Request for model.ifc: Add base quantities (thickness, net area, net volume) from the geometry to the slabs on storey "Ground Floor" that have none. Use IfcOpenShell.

First a look at what the model holds.

```python
import ifcopenshell
import ifcopenshell.util.element
import ifcopenshell.util.unit

model = ifcopenshell.open("model.ifc")
print(model.schema)
for unit_type in ("LENGTHUNIT", "AREAUNIT", "VOLUMEUNIT"):
    print(unit_type, ifcopenshell.util.unit.calculate_unit_scale(model, unit_type))
storey = next(s for s in model.by_type("IfcBuildingStorey") if s.Name == "Ground Floor")
slabs = [e for e in ifcopenshell.util.element.get_decomposition(storey) if e.is_a("IfcSlab")]
for e in sorted(slabs, key=lambda e: e.id()):
    print(e.id(), e.is_a(), e.Name, list(ifcopenshell.util.element.get_psets(e, qtos_only=True)), sep=" | ")
```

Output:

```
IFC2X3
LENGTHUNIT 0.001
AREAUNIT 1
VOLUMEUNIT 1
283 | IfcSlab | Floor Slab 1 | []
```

```python
import ifcopenshell
import ifcopenshell.api.pset
import ifcopenshell.geom
import ifcopenshell.util.element
import ifcopenshell.util.shape
import ifcopenshell.util.unit

model = ifcopenshell.open("model.ifc")
unit_scale = ifcopenshell.util.unit.calculate_unit_scale(model)
area_scale = ifcopenshell.util.unit.calculate_unit_scale(model, "AREAUNIT")
volume_scale = ifcopenshell.util.unit.calculate_unit_scale(model, "VOLUMEUNIT")
settings = ifcopenshell.geom.settings()

storey = next(s for s in model.by_type("IfcBuildingStorey") if s.Name == "Ground Floor")
slabs = [e for e in ifcopenshell.util.element.get_decomposition(storey) if e.is_a("IfcSlab")]

for e in sorted(slabs, key=lambda e: e.id()):
    if ifcopenshell.util.element.get_psets(e, qtos_only=True, should_inherit=False):
        continue
    # Geometry comes back in metres, in the element's own axes.
    shape = ifcopenshell.geom.create_shape(settings, e)
    values = {
        "Width": ifcopenshell.util.shape.get_z(shape.geometry) / unit_scale,
        "NetArea": ifcopenshell.util.shape.get_footprint_area(shape.geometry) / area_scale,
        "NetVolume": ifcopenshell.util.shape.get_volume(shape.geometry) / volume_scale,
    }
    qto = ifcopenshell.api.pset.add_qto(model, product=e, name="BaseQuantities")
    ifcopenshell.api.pset.edit_qto(model, qto=qto, properties=values)
    print(e.id(), {k: round(v, 3) for k, v in values.items()})

model.write("model_v2.ifc")
```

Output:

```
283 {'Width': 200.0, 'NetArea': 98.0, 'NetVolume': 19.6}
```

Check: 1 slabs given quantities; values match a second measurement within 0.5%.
